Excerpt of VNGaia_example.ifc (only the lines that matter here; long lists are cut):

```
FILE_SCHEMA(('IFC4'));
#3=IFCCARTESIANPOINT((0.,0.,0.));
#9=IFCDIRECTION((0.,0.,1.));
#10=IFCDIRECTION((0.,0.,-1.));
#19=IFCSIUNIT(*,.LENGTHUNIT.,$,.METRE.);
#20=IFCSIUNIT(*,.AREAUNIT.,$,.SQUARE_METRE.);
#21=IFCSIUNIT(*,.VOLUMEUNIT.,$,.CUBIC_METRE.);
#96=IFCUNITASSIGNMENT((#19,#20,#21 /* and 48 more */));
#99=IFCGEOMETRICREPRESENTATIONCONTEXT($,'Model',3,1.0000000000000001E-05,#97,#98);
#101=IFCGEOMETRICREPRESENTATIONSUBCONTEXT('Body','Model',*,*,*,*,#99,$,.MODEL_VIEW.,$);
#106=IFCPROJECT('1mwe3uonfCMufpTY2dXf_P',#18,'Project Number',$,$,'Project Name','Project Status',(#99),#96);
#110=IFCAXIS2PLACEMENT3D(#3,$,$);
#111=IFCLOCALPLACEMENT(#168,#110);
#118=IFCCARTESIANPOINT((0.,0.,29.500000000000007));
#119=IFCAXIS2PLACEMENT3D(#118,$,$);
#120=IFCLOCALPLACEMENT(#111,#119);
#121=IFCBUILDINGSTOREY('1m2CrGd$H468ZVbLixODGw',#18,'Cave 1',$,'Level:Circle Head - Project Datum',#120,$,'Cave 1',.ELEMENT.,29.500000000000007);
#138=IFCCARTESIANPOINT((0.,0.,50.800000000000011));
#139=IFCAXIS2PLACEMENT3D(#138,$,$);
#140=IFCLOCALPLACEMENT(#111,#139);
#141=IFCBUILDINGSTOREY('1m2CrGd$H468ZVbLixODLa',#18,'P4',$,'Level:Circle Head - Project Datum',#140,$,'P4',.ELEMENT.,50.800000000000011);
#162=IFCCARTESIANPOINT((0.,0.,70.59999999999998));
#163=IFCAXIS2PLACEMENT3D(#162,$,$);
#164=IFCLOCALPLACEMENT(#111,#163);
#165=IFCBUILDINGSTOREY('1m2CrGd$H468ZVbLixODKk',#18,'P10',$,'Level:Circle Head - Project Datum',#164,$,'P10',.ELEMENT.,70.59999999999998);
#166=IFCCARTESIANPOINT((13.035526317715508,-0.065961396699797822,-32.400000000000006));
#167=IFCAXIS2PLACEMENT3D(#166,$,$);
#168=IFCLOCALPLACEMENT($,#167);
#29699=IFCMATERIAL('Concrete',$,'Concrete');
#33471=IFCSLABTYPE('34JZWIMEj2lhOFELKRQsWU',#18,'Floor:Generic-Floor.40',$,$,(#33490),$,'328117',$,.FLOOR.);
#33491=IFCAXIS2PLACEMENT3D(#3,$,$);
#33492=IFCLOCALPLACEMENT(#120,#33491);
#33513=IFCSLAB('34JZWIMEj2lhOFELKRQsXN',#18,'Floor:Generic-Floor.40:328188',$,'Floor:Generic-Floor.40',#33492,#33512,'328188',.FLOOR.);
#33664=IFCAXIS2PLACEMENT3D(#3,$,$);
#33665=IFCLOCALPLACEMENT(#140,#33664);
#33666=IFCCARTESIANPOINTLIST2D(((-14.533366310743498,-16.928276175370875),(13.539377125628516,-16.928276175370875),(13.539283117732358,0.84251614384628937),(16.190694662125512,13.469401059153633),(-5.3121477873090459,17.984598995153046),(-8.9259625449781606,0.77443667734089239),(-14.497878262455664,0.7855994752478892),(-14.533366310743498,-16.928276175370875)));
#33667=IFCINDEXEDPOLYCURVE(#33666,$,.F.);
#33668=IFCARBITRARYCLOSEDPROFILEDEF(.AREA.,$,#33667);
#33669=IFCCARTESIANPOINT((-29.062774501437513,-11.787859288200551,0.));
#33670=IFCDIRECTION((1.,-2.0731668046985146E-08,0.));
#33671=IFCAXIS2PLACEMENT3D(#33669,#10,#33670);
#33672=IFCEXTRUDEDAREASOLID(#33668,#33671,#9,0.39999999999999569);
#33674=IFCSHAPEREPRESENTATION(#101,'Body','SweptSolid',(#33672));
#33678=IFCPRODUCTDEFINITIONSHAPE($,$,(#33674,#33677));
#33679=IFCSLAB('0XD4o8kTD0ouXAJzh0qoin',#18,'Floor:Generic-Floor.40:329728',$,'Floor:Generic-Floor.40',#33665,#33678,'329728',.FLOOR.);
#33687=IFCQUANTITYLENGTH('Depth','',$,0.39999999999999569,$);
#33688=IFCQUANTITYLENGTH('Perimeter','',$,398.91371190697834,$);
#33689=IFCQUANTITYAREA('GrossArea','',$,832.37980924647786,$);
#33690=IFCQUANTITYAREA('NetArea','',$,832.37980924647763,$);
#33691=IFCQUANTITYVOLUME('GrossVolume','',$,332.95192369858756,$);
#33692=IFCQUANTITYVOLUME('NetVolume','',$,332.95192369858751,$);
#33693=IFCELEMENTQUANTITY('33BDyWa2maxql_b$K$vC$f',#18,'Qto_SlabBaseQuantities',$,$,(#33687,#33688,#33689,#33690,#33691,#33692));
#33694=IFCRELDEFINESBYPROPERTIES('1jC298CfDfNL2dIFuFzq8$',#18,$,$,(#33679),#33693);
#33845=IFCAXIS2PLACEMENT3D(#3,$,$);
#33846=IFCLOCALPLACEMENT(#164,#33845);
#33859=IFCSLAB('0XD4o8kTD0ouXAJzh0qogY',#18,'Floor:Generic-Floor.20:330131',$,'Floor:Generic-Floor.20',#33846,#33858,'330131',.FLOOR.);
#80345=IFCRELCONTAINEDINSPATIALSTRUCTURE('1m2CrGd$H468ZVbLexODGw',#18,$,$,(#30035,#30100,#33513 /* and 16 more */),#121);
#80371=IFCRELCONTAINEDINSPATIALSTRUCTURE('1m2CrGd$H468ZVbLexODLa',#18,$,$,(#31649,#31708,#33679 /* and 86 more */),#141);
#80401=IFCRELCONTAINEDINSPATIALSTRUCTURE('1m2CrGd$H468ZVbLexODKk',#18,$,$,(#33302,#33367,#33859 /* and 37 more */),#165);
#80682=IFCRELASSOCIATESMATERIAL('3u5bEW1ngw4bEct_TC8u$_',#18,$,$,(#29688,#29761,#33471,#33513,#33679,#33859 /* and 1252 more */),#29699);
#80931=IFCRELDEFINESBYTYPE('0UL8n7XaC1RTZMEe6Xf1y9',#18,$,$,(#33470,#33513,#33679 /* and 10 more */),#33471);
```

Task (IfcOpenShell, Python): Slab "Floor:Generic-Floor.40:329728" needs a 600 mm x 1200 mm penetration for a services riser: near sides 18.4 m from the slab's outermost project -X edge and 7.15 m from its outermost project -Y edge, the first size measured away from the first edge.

```python
import numpy as np
import ifcopenshell
import ifcopenshell.api.feature
import ifcopenshell.api.geometry
import ifcopenshell.api.pset
import ifcopenshell.api.root
import ifcopenshell.geom
import ifcopenshell.util.element
import ifcopenshell.util.placement
import ifcopenshell.util.representation
import ifcopenshell.util.shape
import ifcopenshell.util.unit

model = ifcopenshell.open("VNGaia_example.ifc")
unit_scale = ifcopenshell.util.unit.calculate_unit_scale(model)
area_scale = ifcopenshell.util.unit.calculate_unit_scale(model, "AREAUNIT")
volume_scale = ifcopenshell.util.unit.calculate_unit_scale(model, "VOLUMEUNIT")
settings = ifcopenshell.geom.settings()


def volume(element):
    """Net volume in cubic metres, openings subtracted."""
    shape = ifcopenshell.geom.create_shape(settings, element)
    return ifcopenshell.util.shape.get_volume(shape.geometry)


slab = model.by_guid("0XD4o8kTD0ouXAJzh0qoin")
before = volume(slab)

# Extent in the slab's own axes, in metres. The edges named are its -X and -Y sides.
slab_shape = ifcopenshell.geom.create_shape(settings, slab)
vertices = ifcopenshell.util.shape.get_vertices(slab_shape.geometry)
x_min, y_min, bottom = vertices.min(axis=0)
top = vertices[:, 2].max()

opening = ifcopenshell.api.root.create_entity(model, ifc_class="IfcOpeningElement", name="Services riser opening", predefined_type="OPENING")
context = ifcopenshell.util.representation.get_context(model, "Model", "Body", "MODEL_VIEW")
width, depth = 0.6, 1.2
outline = [(0.0, 0.0), (width, 0.0), (width, depth), (0.0, depth), (0.0, 0.0)]
# Overshoot both faces by 50 mm so the cut is clean.
shape = ifcopenshell.api.geometry.add_slab_representation(
    model, context=context, depth=top - bottom + 0.1, polyline=outline
)
ifcopenshell.api.geometry.assign_representation(model, product=opening, representation=shape)

matrix = ifcopenshell.util.placement.get_local_placement(slab.ObjectPlacement)
matrix[:, 3] = matrix @ np.append(np.array([x_min + 18.4, y_min + 7.15, bottom - 0.05]) / unit_scale, 1.0)
ifcopenshell.api.geometry.edit_object_placement(model, product=opening, matrix=matrix, is_si=False)
ifcopenshell.api.feature.add_feature(model, feature=opening, element=slab)

after = volume(slab)

# Update the slab's stored quantities.
qto = model.by_id(ifcopenshell.util.element.get_pset(slab, "Qto_SlabBaseQuantities", should_inherit=False)["id"])
ifcopenshell.api.pset.edit_qto(model, qto=qto, properties={
    "NetArea": after / (top - bottom) / area_scale,
    "NetVolume": after / volume_scale,
})

print(f"slab volume {before:.3f} -> {after:.3f} m3")

model.write("VNGaia_example-out.ifc")
```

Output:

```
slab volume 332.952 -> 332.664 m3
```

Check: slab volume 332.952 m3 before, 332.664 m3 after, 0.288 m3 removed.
